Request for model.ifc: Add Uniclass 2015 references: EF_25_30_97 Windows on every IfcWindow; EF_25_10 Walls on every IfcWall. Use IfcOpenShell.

First a look at what the model holds.

```python
import ifcopenshell

model = ifcopenshell.open("model.ifc")
print(model.schema)
print("classifications:", [c.Name for c in model.by_type("IfcClassification")])
for ifc_class in ("IfcDoor", "IfcRoof", "IfcStair", "IfcWall", "IfcWindow"):
    print(ifc_class, len(model.by_type(ifc_class)))
```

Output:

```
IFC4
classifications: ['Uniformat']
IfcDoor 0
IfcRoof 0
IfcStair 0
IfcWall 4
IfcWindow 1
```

```python
import ifcopenshell
import ifcopenshell.api.classification

model = ifcopenshell.open("model.ifc")

system = ifcopenshell.api.classification.add_classification(model, classification="Uniclass 2015")

codes = {
    "IfcWindow": ("EF_25_30_97", "Windows"),
    "IfcWall": ("EF_25_10", "Walls"),
}
for ifc_class, (code, name) in codes.items():
    products = model.by_type(ifc_class)
    ifcopenshell.api.classification.add_reference(
        model, products=products, classification=system, identification=code, name=name
    )
    print(code, len(products))

model.write("model_v2.ifc")
```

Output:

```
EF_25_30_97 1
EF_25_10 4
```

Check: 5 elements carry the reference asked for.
